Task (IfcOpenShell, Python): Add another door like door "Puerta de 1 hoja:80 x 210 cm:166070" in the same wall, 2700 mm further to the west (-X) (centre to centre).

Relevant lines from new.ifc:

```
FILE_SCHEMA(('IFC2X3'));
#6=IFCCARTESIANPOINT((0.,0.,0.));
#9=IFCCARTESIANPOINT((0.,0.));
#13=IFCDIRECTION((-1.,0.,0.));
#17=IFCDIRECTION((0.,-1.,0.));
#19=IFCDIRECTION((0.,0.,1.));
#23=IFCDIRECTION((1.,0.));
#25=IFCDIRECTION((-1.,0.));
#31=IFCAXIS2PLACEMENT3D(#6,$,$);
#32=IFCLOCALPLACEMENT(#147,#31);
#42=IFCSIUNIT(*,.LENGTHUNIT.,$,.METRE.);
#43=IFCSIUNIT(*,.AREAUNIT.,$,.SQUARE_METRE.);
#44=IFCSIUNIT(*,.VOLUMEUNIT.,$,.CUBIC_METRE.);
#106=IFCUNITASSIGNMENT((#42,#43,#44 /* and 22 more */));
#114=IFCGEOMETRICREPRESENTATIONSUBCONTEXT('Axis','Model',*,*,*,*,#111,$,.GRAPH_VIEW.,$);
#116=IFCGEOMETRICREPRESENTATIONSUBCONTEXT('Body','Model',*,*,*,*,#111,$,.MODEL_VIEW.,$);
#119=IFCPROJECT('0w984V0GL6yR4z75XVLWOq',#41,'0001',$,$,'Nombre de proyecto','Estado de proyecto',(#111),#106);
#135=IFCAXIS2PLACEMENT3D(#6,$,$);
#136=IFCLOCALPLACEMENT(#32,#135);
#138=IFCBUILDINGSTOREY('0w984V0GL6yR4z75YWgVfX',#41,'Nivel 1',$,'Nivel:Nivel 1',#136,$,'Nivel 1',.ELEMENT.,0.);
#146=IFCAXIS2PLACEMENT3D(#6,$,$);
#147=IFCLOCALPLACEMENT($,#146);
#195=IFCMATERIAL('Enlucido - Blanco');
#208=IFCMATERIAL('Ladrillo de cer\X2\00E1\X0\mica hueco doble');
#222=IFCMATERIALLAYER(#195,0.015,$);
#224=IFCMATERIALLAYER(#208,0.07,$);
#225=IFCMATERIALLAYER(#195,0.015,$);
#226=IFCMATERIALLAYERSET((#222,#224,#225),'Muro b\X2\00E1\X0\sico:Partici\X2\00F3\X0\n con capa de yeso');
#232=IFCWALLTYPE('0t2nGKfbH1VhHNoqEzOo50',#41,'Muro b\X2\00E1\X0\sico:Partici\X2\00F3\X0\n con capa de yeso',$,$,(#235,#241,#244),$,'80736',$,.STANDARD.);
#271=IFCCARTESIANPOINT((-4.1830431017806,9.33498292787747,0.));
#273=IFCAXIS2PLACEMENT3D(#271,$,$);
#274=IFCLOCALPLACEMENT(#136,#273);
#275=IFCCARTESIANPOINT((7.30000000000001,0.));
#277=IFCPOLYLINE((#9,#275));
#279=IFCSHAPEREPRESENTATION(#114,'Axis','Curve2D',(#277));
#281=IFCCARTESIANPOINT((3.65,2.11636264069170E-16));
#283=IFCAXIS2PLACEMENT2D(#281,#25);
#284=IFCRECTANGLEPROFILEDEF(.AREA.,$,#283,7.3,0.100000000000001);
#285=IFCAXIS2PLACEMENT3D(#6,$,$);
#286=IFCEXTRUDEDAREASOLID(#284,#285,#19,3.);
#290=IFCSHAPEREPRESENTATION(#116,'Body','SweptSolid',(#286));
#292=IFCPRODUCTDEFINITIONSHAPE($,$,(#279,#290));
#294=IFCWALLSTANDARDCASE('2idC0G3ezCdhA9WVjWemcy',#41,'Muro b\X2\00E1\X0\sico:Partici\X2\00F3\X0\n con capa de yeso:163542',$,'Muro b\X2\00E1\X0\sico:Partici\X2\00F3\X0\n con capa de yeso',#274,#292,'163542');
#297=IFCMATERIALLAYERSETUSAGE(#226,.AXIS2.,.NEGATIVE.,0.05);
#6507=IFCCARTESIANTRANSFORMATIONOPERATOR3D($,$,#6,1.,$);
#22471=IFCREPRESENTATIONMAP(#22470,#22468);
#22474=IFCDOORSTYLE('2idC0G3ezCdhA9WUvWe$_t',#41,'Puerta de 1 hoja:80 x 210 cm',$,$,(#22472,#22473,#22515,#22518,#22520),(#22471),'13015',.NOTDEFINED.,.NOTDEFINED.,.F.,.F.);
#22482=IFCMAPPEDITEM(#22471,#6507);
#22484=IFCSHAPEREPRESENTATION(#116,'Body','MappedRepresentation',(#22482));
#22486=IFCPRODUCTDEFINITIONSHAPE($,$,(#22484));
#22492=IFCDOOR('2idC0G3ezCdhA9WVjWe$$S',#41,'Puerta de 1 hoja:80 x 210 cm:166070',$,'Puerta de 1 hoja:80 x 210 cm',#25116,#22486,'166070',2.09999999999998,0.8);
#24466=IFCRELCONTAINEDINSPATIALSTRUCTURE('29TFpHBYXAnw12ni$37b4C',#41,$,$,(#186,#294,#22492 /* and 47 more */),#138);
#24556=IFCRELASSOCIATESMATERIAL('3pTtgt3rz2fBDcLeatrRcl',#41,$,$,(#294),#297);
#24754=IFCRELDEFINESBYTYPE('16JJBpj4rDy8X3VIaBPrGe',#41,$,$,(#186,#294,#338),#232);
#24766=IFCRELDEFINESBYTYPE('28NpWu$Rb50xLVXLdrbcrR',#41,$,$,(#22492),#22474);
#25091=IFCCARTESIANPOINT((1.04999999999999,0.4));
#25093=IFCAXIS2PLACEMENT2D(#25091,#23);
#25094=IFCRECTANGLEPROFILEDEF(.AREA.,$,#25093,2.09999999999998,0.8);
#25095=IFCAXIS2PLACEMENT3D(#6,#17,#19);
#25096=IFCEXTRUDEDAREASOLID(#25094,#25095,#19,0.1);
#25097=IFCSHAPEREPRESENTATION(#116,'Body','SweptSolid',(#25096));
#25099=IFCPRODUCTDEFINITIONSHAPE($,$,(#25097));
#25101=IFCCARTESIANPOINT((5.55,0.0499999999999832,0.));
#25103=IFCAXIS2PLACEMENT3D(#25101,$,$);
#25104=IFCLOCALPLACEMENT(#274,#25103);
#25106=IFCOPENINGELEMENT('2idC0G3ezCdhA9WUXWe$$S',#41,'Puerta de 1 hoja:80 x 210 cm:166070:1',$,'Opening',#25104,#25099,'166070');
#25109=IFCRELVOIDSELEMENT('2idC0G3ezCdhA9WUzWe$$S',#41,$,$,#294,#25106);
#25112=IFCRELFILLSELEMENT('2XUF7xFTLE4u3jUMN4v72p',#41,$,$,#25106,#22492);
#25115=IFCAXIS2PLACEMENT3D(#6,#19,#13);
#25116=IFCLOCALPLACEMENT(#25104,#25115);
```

```python
import ifcopenshell
import ifcopenshell.api.feature
import ifcopenshell.api.geometry
import ifcopenshell.api.root
import ifcopenshell.geom
import ifcopenshell.util.element
import ifcopenshell.util.placement
import ifcopenshell.util.shape
import ifcopenshell.util.unit

model = ifcopenshell.open("new.ifc")
unit_scale = ifcopenshell.util.unit.calculate_unit_scale(model)
settings = ifcopenshell.geom.settings()


def volume(element):
    """Net volume in cubic metres, openings subtracted."""
    shape = ifcopenshell.geom.create_shape(settings, element)
    return ifcopenshell.util.shape.get_volume(shape.geometry)


def reuse_history(source, copy):
    """copy_class also copies each property set's owner history, people and application; keep the originals."""
    for rel in copy.IsDefinedBy:
        if rel.is_a("IfcRelDefinesByProperties") and (history := rel.RelatingPropertyDefinition.OwnerHistory):
            rel.RelatingPropertyDefinition.OwnerHistory = source.OwnerHistory
            ifcopenshell.util.element.remove_deep2(model, history)


door = model.by_guid("2idC0G3ezCdhA9WVjWe$$S")
opening = door.FillsVoids[0].RelatingOpeningElement
wall = opening.VoidsElements[0].RelatingBuildingElement
before = volume(wall)
shift = ifcopenshell.util.placement.get_local_placement(wall.ObjectPlacement)[:3, 0] * -2.7 / unit_scale

# copy_class copies the void relationship, type, container and properties, but no geometry.
new_opening = ifcopenshell.api.root.copy_class(model, product=opening)
new_opening.Representation = ifcopenshell.util.element.copy_deep(
    model, opening.Representation, exclude=["IfcGeometricRepresentationContext", "IfcRepresentationMap"]
)
new_opening.Name = "Puerta de 1 hoja:80 x 210 cm"
new_opening.Tag = None
new_door = ifcopenshell.api.root.copy_class(model, product=door)
new_door.Representation = ifcopenshell.util.element.copy_deep(
    model, door.Representation, exclude=["IfcGeometricRepresentationContext", "IfcRepresentationMap"]
)
new_door.Name = "Puerta de 1 hoja:80 x 210 cm"
new_door.Tag = None
reuse_history(door, new_door)
fills = ifcopenshell.api.feature.add_filling(model, opening=new_opening, element=new_door)
fills.OwnerHistory = new_door.OwnerHistory  # required in IFC2X3

for old, new in ((opening, new_opening), (door, new_door)):
    matrix = ifcopenshell.util.placement.get_local_placement(old.ObjectPlacement)
    matrix[:3, 3] += shift
    ifcopenshell.api.geometry.edit_object_placement(model, product=new, matrix=matrix, is_si=False)

after = volume(wall)

print(f"wall volume {before:.3f} -> {after:.3f} m3")

model.write("new_v2.ifc")
```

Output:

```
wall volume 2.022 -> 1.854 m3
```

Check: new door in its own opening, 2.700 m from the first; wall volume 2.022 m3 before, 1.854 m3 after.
